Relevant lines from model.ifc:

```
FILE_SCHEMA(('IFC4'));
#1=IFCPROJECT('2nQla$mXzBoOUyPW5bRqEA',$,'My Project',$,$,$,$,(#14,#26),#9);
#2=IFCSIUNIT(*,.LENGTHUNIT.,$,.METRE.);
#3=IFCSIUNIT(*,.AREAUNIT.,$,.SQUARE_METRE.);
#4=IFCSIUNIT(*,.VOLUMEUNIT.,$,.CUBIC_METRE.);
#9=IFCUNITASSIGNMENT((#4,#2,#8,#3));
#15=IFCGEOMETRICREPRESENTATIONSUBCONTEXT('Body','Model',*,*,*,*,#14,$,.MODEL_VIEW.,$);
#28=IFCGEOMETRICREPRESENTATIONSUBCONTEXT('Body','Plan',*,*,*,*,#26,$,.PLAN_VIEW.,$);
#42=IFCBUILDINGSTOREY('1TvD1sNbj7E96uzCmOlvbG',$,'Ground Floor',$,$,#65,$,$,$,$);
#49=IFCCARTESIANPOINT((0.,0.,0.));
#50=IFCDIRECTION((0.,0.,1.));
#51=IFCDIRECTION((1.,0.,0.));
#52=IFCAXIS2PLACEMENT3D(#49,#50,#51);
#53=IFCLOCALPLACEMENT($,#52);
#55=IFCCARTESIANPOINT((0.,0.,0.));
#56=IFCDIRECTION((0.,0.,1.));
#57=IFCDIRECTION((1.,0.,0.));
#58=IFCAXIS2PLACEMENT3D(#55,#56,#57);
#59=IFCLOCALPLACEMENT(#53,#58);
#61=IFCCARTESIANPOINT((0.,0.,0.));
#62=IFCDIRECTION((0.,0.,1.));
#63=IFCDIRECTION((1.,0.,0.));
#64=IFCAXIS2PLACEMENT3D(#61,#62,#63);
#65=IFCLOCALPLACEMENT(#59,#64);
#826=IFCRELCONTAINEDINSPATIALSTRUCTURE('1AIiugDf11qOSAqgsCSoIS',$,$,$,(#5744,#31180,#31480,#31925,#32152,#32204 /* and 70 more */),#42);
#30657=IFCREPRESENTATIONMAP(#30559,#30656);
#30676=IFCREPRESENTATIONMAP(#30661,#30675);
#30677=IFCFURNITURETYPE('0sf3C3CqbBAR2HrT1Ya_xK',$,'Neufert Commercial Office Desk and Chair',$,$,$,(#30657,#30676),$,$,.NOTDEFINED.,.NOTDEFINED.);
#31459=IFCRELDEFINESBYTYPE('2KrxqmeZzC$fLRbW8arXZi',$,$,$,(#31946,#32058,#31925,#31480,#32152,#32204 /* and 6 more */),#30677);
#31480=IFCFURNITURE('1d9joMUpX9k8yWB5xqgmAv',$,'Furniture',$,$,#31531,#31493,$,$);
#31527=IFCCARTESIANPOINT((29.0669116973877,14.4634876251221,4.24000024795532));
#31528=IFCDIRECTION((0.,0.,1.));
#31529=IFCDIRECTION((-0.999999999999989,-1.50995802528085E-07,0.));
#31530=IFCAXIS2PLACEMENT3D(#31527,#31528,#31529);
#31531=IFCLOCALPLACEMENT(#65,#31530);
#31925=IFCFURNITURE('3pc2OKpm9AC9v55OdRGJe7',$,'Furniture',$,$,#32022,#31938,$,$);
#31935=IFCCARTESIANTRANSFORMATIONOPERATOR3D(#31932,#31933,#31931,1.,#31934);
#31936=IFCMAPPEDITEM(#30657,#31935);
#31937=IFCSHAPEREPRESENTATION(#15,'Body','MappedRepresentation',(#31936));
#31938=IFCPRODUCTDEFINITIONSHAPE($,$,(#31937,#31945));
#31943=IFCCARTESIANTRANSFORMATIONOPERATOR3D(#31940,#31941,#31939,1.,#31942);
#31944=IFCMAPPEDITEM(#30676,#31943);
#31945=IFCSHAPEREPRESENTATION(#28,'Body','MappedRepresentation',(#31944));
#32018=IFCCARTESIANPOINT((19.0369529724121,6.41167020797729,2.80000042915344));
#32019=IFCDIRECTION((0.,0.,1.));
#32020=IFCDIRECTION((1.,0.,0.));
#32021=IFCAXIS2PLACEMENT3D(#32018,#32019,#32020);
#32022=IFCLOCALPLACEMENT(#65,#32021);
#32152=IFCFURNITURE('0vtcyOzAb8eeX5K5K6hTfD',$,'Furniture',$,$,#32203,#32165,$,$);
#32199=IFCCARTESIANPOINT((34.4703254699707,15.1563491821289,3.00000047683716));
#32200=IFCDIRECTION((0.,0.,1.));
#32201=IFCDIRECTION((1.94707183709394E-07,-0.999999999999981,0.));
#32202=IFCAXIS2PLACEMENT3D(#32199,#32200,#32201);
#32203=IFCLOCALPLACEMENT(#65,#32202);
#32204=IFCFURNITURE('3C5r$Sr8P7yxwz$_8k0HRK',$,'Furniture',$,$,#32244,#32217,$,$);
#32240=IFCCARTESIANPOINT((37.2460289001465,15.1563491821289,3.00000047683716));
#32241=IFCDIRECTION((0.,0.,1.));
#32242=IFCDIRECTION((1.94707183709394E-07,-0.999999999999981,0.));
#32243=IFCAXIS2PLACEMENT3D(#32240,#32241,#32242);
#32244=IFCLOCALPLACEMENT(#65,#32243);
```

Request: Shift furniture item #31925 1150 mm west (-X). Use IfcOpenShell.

```python
import ifcopenshell
import ifcopenshell.api.geometry
import ifcopenshell.util.placement
import ifcopenshell.util.unit

model = ifcopenshell.open("model.ifc")
unit_scale = ifcopenshell.util.unit.calculate_unit_scale(model)

item = model.by_guid("3pc2OKpm9AC9v55OdRGJe7")
matrix = ifcopenshell.util.placement.get_local_placement(item.ObjectPlacement)
matrix[0, 3] -= 1.15 / unit_scale
ifcopenshell.api.geometry.edit_object_placement(model, product=item, matrix=matrix, is_si=False)

print(ifcopenshell.util.placement.get_local_placement(item.ObjectPlacement).round(3) + 0.0)

model.write("model_updated.ifc")
```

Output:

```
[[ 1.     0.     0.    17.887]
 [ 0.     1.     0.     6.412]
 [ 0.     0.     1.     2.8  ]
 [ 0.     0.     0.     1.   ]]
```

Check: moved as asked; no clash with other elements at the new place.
